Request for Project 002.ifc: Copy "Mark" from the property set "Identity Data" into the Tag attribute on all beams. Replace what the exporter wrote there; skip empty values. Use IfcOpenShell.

First a look at what the model holds.

```python
import ifcopenshell
import ifcopenshell.util.element

model = ifcopenshell.open("Project 002.ifc")
print(model.schema)
beams = model.by_type("IfcBeam")
print(len(beams), "beams")
for e in beams[:8]:
    source = ifcopenshell.util.element.get_pset(e, "Identity Data", "Mark")
    target = e.Tag
    print(e.id(), repr(source), repr(target), sep=" | ")
```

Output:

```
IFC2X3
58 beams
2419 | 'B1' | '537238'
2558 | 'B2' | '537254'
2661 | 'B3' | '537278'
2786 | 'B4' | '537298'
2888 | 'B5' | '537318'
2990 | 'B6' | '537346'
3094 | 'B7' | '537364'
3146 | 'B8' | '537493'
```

```python
import ifcopenshell
import ifcopenshell.util.element

model = ifcopenshell.open("Project 002.ifc")

count = 0
for e in model.by_type("IfcBeam"):
    value = ifcopenshell.util.element.get_pset(e, "Identity Data", "Mark")
    current = e.Tag
    if not value or not value.strip() or current == value:
        continue
    e.Tag = value
    count += 1

print(count, "beams updated")

model.write("Project 002_v2.ifc")
```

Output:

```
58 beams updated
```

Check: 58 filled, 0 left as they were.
